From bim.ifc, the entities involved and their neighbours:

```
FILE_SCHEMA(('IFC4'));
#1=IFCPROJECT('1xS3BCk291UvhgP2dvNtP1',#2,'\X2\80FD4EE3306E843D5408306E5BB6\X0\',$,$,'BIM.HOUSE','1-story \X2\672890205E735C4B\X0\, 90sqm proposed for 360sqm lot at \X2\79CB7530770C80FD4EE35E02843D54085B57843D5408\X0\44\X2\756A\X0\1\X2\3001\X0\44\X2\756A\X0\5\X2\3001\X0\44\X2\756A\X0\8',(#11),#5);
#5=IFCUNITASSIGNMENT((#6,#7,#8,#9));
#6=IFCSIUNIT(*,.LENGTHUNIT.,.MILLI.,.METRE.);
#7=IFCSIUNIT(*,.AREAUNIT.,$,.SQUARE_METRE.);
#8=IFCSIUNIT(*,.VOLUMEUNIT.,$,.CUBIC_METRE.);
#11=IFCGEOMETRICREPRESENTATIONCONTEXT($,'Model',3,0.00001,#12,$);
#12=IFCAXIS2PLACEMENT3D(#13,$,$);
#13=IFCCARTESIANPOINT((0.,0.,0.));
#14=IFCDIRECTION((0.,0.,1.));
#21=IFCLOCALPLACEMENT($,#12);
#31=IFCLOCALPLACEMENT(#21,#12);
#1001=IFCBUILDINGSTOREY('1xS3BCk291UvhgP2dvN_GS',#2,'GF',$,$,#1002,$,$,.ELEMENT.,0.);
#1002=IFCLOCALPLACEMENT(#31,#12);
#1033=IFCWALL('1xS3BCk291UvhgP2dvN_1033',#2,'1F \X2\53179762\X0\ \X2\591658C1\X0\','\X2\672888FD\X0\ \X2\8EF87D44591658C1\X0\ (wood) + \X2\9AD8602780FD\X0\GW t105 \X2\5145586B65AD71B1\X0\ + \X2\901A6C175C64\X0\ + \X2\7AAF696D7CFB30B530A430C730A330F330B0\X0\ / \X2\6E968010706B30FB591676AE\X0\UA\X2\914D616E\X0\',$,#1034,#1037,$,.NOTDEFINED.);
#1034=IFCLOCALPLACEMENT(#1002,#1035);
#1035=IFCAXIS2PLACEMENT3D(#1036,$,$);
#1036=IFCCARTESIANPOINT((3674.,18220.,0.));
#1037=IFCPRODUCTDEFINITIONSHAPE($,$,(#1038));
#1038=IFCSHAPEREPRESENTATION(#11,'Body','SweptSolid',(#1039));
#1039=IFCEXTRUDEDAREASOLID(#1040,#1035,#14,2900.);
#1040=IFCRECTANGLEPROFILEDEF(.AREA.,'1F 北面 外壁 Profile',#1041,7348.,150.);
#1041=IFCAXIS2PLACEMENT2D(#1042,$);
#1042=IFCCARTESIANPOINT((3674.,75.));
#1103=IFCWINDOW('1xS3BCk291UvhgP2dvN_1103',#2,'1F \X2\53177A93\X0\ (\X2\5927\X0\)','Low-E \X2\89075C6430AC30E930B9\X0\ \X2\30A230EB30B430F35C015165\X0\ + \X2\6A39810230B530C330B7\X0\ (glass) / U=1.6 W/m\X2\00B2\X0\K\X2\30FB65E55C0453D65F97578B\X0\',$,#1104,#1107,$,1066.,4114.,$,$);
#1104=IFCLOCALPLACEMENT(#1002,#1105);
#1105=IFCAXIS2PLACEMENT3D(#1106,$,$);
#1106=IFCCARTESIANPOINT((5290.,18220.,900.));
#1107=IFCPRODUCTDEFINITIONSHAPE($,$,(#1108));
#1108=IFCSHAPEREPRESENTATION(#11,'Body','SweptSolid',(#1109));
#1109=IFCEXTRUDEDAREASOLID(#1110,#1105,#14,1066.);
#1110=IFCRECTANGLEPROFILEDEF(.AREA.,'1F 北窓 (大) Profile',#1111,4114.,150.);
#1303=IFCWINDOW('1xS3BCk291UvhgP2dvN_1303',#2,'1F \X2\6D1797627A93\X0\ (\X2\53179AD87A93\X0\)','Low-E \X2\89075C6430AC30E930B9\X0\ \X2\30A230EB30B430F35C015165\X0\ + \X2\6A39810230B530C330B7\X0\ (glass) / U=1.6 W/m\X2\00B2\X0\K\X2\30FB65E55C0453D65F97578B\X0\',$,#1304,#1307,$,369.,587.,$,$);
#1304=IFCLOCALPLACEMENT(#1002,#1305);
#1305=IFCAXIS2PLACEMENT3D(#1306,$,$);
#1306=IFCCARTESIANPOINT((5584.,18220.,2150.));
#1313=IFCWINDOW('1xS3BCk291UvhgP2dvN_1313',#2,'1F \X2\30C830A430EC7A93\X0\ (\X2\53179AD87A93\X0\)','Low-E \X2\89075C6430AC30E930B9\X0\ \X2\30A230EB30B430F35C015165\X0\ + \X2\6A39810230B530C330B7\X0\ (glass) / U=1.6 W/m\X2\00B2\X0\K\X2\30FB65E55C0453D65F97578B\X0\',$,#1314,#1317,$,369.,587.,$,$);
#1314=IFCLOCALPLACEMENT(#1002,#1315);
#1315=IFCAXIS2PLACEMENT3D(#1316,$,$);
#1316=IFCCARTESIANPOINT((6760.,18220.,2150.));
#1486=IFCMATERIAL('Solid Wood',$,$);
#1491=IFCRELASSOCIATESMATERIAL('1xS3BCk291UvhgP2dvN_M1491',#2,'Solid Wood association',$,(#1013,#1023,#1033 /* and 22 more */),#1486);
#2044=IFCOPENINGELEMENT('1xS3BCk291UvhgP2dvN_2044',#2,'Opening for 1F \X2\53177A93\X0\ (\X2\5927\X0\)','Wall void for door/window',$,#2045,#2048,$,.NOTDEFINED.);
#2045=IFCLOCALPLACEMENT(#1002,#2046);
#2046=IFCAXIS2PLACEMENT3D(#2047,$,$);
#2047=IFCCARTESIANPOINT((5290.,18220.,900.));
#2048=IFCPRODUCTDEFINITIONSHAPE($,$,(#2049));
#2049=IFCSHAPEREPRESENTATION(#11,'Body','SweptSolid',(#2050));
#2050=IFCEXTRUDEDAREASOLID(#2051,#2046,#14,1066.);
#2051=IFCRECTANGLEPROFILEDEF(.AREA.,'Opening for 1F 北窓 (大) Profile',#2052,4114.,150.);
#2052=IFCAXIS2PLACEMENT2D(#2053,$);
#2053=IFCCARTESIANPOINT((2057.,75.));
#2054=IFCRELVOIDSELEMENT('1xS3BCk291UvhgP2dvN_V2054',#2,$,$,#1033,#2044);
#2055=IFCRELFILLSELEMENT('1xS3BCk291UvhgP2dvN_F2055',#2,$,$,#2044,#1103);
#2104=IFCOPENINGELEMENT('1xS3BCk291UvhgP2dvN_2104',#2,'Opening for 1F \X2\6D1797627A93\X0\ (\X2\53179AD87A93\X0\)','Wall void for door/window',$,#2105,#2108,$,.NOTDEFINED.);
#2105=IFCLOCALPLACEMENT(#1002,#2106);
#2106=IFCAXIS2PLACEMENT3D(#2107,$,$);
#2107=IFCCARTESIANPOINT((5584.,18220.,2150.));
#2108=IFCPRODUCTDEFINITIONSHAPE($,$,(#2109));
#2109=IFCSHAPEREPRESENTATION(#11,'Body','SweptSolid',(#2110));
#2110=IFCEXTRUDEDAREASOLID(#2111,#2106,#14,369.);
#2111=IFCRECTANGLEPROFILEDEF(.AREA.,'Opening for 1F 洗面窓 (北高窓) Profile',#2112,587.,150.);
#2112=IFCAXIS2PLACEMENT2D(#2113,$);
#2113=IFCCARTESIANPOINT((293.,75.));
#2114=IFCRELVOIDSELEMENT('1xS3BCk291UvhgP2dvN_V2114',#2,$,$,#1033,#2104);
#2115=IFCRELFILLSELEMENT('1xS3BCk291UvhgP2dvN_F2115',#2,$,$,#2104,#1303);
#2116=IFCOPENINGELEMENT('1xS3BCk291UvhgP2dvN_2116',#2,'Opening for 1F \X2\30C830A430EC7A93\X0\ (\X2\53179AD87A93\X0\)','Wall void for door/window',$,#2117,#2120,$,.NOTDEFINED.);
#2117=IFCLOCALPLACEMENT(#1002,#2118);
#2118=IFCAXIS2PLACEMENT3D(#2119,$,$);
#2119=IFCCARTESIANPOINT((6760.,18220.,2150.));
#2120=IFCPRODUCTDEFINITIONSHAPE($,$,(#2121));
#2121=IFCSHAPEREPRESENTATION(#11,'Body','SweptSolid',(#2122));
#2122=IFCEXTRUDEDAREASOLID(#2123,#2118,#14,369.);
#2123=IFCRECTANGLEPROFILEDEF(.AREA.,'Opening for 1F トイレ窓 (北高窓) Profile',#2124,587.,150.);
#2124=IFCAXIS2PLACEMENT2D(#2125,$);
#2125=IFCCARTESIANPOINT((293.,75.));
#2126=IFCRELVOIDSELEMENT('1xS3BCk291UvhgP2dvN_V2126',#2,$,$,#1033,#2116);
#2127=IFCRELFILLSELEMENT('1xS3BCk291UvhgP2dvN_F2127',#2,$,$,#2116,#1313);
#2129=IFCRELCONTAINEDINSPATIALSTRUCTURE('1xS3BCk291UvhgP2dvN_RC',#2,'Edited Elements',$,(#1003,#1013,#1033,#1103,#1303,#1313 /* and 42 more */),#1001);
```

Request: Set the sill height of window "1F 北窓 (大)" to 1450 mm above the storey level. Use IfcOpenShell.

```python
import numpy as np
import ifcopenshell
import ifcopenshell.api.geometry
import ifcopenshell.geom
import ifcopenshell.util.element
import ifcopenshell.util.placement
import ifcopenshell.util.shape
import ifcopenshell.util.unit

model = ifcopenshell.open("bim.ifc")
unit_scale = ifcopenshell.util.unit.calculate_unit_scale(model)

window = model.by_id(1103)
opening = window.FillsVoids[0].RelatingOpeningElement
storey = ifcopenshell.util.element.get_container(window, ifc_class="IfcBuildingStorey")
level = ifcopenshell.util.placement.get_local_placement(storey.ObjectPlacement)[2, 3]

# The opening's origin need not be at the sill, so measure its lowest point.
shape = ifcopenshell.geom.create_shape(ifcopenshell.geom.settings(), opening)
bottom = ifcopenshell.util.shape.get_shape_bottom_elevation(shape, shape.geometry) / unit_scale
dz = level + 1.45 / unit_scale - bottom

shift = np.array([0.0, 0.0, dz])
# The window is not placed relative to its opening, so move both.
for product in (opening, window):
    matrix = ifcopenshell.util.placement.get_local_placement(product.ObjectPlacement)
    matrix[:3, 3] += shift
    ifcopenshell.api.geometry.edit_object_placement(model, product=product, matrix=matrix, is_si=False)

print(f"moved by {dz * unit_scale:+.3f} m")

model.write("bim-out.ifc")
```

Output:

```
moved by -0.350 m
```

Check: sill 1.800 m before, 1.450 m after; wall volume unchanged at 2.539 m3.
